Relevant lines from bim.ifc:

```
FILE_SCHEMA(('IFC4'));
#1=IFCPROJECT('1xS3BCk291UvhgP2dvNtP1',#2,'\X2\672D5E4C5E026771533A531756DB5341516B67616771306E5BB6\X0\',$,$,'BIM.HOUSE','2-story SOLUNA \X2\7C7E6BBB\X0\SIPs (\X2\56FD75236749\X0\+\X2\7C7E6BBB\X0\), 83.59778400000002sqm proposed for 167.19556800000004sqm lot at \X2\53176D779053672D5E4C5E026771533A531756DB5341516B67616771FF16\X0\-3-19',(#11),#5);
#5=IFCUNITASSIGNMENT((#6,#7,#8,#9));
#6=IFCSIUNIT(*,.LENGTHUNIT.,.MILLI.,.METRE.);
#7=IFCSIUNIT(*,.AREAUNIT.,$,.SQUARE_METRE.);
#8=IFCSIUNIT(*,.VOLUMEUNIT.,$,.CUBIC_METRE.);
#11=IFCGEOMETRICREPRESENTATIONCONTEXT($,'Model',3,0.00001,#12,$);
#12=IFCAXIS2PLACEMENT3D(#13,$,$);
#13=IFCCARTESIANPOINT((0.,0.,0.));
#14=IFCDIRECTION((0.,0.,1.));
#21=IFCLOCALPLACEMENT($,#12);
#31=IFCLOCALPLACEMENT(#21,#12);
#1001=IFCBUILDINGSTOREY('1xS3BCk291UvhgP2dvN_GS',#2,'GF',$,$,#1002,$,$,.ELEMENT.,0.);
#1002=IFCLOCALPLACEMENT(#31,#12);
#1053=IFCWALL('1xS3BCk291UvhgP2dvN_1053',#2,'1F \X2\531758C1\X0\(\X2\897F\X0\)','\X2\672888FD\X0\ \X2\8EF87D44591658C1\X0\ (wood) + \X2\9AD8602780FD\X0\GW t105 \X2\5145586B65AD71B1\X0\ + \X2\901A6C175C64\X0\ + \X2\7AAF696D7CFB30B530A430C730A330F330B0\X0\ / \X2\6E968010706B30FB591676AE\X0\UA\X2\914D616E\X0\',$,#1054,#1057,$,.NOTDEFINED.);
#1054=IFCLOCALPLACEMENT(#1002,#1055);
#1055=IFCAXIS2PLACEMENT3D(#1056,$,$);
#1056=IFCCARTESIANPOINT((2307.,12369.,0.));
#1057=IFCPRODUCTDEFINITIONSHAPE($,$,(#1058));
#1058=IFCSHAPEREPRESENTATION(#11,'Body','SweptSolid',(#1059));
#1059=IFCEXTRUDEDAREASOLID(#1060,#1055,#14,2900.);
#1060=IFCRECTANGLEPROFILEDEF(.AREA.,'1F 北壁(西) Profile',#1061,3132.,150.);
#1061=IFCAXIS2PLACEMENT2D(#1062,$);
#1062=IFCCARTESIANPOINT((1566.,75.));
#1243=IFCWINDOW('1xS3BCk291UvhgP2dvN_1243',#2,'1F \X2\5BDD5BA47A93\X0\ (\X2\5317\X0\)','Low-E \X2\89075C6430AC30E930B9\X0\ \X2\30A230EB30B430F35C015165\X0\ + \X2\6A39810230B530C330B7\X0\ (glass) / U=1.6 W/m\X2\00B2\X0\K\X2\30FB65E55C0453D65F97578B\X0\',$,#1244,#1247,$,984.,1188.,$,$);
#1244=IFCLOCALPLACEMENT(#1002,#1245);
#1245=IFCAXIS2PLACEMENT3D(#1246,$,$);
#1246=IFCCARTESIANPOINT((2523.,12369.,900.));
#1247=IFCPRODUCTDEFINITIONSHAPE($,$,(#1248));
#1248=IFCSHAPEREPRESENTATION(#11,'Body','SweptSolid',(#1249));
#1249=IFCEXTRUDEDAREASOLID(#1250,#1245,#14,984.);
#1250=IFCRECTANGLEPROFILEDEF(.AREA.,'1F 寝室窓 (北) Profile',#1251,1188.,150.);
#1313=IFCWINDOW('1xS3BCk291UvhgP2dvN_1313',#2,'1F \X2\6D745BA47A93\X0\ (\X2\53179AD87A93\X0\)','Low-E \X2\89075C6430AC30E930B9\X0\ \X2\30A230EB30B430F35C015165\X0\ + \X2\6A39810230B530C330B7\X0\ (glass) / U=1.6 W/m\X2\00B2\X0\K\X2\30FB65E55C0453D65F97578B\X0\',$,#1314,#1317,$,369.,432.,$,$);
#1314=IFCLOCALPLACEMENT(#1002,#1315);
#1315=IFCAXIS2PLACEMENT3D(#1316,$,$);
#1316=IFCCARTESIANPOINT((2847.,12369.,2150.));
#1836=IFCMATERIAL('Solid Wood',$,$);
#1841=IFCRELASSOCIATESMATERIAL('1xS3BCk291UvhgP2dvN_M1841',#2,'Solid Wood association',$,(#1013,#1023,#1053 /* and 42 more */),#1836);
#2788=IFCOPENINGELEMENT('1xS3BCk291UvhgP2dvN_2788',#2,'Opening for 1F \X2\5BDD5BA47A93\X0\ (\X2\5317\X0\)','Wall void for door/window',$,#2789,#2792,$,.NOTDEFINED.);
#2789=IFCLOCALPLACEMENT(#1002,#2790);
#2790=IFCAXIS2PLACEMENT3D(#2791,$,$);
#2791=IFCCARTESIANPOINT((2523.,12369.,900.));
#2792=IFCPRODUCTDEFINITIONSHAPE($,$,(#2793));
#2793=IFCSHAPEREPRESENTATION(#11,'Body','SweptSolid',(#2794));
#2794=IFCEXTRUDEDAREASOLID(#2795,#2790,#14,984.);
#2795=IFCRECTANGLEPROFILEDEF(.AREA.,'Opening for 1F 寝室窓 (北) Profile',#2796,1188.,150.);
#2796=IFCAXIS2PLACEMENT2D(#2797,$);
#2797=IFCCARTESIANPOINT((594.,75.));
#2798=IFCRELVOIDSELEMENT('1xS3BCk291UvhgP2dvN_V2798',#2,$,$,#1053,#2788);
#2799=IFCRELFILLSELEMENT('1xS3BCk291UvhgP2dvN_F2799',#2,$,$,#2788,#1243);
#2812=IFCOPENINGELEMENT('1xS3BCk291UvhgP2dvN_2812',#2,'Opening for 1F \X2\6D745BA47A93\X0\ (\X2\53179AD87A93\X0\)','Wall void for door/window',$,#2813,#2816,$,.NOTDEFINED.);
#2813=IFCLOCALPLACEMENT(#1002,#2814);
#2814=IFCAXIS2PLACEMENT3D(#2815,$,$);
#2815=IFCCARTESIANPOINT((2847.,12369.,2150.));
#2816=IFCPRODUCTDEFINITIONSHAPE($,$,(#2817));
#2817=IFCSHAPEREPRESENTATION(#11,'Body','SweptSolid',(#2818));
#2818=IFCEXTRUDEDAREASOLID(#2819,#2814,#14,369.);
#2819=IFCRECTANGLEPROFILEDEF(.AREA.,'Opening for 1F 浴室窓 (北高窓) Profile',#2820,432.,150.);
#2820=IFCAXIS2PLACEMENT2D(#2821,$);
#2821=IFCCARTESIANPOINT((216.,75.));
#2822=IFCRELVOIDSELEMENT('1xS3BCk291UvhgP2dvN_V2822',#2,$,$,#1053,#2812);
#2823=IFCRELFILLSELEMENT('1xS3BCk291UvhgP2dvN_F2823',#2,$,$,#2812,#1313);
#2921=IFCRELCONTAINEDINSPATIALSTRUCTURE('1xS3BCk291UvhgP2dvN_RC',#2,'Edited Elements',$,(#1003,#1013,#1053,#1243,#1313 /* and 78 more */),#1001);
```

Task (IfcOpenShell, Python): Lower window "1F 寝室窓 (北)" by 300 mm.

```python
import numpy as np
import ifcopenshell
import ifcopenshell.api.geometry
import ifcopenshell.util.placement
import ifcopenshell.util.unit

model = ifcopenshell.open("bim.ifc")
unit_scale = ifcopenshell.util.unit.calculate_unit_scale(model)

window = model.by_guid("1xS3BCk291UvhgP2dvN_1243")
opening = window.FillsVoids[0].RelatingOpeningElement
dz = -0.3 / unit_scale

shift = np.array([0.0, 0.0, dz])
# The window is not placed relative to its opening, so move both.
for product in (opening, window):
    matrix = ifcopenshell.util.placement.get_local_placement(product.ObjectPlacement)
    matrix[:3, 3] += shift
    ifcopenshell.api.geometry.edit_object_placement(model, product=product, matrix=matrix, is_si=False)

print(f"moved by {dz * unit_scale:+.3f} m")

model.write("bim_edited.ifc")
```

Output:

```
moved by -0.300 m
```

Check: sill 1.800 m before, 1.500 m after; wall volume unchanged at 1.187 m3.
